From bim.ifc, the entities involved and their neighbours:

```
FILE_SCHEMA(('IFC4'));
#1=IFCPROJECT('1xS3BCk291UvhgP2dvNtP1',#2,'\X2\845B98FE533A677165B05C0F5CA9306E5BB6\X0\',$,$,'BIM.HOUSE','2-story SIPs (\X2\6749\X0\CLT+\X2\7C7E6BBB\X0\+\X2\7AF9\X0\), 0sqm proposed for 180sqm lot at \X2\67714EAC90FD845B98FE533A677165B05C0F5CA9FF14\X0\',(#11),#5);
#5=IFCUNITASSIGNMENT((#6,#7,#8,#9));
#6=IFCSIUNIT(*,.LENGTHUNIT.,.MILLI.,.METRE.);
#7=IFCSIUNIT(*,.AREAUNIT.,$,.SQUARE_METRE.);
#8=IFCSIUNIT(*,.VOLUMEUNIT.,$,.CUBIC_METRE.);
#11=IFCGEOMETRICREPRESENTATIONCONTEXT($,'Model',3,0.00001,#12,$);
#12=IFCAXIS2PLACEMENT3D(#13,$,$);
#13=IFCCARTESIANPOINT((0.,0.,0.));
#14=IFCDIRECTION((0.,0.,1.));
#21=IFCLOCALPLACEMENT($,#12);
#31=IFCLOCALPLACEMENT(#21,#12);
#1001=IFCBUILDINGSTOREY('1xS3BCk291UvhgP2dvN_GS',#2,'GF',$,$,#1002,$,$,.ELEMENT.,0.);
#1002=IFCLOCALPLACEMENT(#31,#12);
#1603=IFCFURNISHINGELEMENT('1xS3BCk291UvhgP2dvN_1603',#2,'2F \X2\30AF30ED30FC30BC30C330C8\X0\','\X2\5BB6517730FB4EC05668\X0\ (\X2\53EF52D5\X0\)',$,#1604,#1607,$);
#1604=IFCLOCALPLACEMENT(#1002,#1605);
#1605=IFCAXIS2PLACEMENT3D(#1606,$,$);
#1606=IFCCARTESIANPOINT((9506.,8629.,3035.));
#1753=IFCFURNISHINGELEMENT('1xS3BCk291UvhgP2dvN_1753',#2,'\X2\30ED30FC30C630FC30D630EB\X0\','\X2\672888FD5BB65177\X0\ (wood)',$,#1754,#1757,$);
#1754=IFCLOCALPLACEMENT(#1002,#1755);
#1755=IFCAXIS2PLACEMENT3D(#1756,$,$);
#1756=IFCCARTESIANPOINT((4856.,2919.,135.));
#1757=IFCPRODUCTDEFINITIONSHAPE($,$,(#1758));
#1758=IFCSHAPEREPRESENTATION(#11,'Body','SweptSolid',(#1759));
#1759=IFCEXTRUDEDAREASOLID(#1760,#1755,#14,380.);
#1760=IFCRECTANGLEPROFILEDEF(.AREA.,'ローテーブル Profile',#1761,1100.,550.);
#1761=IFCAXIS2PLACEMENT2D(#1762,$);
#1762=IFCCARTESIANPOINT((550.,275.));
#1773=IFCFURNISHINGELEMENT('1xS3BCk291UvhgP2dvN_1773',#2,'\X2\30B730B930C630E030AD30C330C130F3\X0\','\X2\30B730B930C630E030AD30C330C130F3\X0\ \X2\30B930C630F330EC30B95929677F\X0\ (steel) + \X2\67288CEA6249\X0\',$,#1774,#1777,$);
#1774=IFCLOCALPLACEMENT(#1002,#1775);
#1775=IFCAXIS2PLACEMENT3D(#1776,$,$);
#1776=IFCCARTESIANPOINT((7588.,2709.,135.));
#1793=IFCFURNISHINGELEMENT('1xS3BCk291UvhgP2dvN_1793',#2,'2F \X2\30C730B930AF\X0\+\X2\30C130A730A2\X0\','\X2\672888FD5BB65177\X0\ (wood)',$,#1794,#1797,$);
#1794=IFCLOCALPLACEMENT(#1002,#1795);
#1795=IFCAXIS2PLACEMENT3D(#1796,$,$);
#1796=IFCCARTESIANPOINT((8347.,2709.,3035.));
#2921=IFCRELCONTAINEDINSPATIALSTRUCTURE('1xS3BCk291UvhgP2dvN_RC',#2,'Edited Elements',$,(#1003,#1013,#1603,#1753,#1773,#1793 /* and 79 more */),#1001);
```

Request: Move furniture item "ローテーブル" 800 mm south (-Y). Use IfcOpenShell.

```python
import ifcopenshell
import ifcopenshell.api.geometry
import ifcopenshell.util.placement
import ifcopenshell.util.unit

model = ifcopenshell.open("bim.ifc")
unit_scale = ifcopenshell.util.unit.calculate_unit_scale(model)

item = model.by_id(1753)
matrix = ifcopenshell.util.placement.get_local_placement(item.ObjectPlacement)
matrix[1, 3] -= 0.8 / unit_scale
ifcopenshell.api.geometry.edit_object_placement(model, product=item, matrix=matrix, is_si=False)

print(ifcopenshell.util.placement.get_local_placement(item.ObjectPlacement).round(3) + 0.0)

model.write("bim_rev.ifc")
```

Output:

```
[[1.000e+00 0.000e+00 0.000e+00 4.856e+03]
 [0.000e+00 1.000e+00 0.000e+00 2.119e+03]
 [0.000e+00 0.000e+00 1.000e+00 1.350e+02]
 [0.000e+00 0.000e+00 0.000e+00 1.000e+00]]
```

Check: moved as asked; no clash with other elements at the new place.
